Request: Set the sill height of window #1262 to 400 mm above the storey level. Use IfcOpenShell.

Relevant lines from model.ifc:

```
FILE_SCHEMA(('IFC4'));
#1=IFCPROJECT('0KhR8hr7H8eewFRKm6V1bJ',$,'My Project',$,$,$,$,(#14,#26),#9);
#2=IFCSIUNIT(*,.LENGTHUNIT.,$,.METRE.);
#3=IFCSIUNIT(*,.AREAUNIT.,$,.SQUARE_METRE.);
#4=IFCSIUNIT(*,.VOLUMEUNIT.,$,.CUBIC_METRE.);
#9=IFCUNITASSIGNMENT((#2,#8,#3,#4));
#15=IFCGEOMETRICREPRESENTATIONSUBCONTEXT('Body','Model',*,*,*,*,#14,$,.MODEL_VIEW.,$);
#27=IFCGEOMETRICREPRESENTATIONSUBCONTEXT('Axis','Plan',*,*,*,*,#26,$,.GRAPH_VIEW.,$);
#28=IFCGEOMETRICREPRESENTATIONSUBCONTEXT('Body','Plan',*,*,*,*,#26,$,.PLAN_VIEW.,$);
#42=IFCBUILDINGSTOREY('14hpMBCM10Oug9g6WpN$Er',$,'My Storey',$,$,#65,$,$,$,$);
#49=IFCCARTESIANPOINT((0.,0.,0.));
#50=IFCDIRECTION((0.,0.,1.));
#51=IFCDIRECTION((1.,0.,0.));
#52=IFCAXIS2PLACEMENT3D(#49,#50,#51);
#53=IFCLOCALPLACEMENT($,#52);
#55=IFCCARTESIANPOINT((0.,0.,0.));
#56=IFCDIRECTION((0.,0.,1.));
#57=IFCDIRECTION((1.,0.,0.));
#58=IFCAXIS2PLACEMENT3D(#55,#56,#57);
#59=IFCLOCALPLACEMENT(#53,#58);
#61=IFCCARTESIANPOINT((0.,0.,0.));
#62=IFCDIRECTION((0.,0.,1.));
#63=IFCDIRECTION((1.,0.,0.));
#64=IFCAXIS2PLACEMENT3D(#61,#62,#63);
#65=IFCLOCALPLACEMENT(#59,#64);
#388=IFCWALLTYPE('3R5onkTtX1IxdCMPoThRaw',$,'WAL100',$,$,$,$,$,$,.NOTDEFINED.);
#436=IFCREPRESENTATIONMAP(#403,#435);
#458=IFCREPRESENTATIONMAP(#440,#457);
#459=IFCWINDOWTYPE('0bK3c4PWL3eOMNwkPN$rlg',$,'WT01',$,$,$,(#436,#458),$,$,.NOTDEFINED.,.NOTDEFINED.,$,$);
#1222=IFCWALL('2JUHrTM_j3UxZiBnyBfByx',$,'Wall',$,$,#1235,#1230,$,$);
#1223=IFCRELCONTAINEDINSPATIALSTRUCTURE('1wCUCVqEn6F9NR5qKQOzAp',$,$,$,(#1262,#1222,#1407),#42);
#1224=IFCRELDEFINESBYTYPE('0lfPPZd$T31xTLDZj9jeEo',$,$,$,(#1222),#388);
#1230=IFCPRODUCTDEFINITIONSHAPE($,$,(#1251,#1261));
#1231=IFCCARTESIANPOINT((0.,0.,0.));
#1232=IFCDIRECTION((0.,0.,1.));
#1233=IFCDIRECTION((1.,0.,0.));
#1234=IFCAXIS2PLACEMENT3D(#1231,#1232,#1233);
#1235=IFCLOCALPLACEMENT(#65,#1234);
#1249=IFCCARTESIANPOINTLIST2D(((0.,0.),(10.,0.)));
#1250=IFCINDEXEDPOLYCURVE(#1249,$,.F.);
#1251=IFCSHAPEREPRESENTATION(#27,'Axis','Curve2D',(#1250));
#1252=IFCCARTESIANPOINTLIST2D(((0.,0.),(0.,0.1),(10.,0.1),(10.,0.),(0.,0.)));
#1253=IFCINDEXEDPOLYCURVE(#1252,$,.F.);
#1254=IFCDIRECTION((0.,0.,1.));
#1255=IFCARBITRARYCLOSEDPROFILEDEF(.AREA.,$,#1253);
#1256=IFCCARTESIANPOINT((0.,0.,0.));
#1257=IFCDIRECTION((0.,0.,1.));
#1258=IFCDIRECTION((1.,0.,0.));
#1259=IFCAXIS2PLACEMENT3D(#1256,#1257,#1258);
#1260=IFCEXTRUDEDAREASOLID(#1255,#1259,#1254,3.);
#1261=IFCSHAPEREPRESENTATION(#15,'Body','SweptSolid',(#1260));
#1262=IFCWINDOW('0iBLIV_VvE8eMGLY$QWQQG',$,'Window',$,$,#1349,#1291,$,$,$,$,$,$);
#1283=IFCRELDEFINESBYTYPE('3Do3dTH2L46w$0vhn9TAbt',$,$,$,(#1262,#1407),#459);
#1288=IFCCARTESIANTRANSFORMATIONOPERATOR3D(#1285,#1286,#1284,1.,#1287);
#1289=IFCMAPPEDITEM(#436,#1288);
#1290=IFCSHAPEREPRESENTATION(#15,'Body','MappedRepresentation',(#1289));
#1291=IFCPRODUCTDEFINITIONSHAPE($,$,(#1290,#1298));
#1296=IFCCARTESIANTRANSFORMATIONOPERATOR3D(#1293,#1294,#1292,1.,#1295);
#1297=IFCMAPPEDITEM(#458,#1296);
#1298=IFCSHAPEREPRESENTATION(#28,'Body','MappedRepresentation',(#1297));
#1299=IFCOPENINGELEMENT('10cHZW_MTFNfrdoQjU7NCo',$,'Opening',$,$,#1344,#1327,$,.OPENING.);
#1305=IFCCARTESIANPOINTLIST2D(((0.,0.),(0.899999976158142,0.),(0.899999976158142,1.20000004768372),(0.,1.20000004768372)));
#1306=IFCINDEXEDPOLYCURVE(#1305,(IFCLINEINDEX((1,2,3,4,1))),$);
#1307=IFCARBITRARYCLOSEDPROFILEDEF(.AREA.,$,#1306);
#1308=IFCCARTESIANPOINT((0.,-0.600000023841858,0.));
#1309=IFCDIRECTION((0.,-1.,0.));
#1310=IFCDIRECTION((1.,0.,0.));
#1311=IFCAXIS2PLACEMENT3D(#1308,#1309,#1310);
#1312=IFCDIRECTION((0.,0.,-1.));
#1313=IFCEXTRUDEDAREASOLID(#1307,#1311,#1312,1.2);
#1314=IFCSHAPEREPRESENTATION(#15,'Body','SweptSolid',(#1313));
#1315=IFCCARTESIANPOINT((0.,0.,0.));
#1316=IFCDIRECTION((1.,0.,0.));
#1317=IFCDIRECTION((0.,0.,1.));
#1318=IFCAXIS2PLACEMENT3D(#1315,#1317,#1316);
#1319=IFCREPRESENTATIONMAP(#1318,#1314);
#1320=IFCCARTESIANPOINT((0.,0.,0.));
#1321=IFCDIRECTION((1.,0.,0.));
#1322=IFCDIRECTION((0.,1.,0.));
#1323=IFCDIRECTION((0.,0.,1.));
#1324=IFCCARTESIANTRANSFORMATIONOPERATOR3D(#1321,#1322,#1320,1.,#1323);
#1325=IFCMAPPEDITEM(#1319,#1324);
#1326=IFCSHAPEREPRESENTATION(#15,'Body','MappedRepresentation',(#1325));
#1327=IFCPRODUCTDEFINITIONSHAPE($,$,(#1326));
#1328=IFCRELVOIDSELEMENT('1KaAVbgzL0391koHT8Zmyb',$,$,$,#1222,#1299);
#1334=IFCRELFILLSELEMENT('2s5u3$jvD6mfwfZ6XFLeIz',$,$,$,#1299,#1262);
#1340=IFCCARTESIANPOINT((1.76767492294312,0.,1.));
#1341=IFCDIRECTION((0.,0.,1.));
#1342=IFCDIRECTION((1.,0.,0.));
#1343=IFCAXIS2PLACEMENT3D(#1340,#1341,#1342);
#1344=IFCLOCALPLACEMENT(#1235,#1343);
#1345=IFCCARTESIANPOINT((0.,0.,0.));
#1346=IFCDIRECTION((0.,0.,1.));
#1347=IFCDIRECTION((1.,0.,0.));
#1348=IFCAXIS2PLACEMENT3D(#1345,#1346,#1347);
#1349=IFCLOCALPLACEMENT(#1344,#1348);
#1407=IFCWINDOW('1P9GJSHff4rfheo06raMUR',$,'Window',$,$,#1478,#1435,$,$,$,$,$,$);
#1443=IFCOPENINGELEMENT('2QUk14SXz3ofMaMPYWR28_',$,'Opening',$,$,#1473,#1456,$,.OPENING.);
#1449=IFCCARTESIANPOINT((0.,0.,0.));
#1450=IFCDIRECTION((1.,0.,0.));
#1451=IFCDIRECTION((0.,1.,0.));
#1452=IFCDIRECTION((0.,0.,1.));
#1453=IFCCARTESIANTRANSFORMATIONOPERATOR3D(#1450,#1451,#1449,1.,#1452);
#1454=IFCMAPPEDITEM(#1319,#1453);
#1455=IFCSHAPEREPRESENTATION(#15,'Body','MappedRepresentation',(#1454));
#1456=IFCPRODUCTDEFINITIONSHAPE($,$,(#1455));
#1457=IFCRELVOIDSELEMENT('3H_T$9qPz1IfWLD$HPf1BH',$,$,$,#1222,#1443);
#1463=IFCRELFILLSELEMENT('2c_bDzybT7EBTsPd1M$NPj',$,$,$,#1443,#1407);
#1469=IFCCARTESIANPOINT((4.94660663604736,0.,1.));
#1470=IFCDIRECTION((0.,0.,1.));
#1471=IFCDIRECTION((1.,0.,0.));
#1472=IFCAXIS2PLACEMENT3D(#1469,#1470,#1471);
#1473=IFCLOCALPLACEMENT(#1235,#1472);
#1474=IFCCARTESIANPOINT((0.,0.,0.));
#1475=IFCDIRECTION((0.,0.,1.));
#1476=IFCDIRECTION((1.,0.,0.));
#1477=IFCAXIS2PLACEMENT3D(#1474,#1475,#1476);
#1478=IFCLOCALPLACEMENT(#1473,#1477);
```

```python
import numpy as np
import ifcopenshell
import ifcopenshell.api.geometry
import ifcopenshell.geom
import ifcopenshell.util.element
import ifcopenshell.util.placement
import ifcopenshell.util.shape
import ifcopenshell.util.unit

model = ifcopenshell.open("model.ifc")
unit_scale = ifcopenshell.util.unit.calculate_unit_scale(model)

window = model.by_id(1262)
opening = window.FillsVoids[0].RelatingOpeningElement
storey = ifcopenshell.util.element.get_container(window, ifc_class="IfcBuildingStorey")
level = ifcopenshell.util.placement.get_local_placement(storey.ObjectPlacement)[2, 3]

# The opening's origin need not be at the sill, so measure its lowest point.
shape = ifcopenshell.geom.create_shape(ifcopenshell.geom.settings(), opening)
bottom = ifcopenshell.util.shape.get_shape_bottom_elevation(shape, shape.geometry) / unit_scale
dz = level + 0.4 / unit_scale - bottom

shift = np.array([0.0, 0.0, dz])
# The window is placed relative to its opening, so it follows when the opening moves.
matrix = ifcopenshell.util.placement.get_local_placement(opening.ObjectPlacement)
matrix[:3, 3] += shift
ifcopenshell.api.geometry.edit_object_placement(
    model, product=opening, matrix=matrix, is_si=False, should_transform_children=True
)

print(f"moved by {dz * unit_scale:+.3f} m")

model.write("model_v2.ifc")
```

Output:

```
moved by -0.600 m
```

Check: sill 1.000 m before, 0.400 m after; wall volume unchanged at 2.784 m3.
